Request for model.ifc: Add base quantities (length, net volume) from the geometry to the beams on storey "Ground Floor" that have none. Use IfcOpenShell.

First a look at what the model holds.

```python
import ifcopenshell
import ifcopenshell.util.element
import ifcopenshell.util.unit

model = ifcopenshell.open("model.ifc")
print(model.schema)
for unit_type in ("LENGTHUNIT", "AREAUNIT", "VOLUMEUNIT"):
    print(unit_type, ifcopenshell.util.unit.calculate_unit_scale(model, unit_type))
storey = next(s for s in model.by_type("IfcBuildingStorey") if s.Name == "Ground Floor")
beams = [e for e in ifcopenshell.util.element.get_decomposition(storey) if e.is_a("IfcBeam")]
for e in sorted(beams, key=lambda e: e.id()):
    print(e.id(), e.is_a(), e.Name, list(ifcopenshell.util.element.get_psets(e, qtos_only=True)), sep=" | ")
```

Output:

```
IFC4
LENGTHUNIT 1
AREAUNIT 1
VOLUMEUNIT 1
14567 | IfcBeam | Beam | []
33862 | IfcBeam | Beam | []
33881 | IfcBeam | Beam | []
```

```python
import ifcopenshell
import ifcopenshell.api.pset
import ifcopenshell.geom
import ifcopenshell.util.element
import ifcopenshell.util.shape
import ifcopenshell.util.unit

model = ifcopenshell.open("model.ifc")
unit_scale = ifcopenshell.util.unit.calculate_unit_scale(model)
volume_scale = ifcopenshell.util.unit.calculate_unit_scale(model, "VOLUMEUNIT")
settings = ifcopenshell.geom.settings()

storey = next(s for s in model.by_type("IfcBuildingStorey") if s.Name == "Ground Floor")
beams = [e for e in ifcopenshell.util.element.get_decomposition(storey) if e.is_a("IfcBeam")]

for e in sorted(beams, key=lambda e: e.id()):
    if ifcopenshell.util.element.get_psets(e, qtos_only=True, should_inherit=False):
        continue
    # Geometry comes back in metres, in the element's own axes.
    shape = ifcopenshell.geom.create_shape(settings, e)
    values = {
        "Length": ifcopenshell.util.shape.get_max_xyz(shape.geometry) / unit_scale,
        "NetVolume": ifcopenshell.util.shape.get_volume(shape.geometry) / volume_scale,
    }
    qto = ifcopenshell.api.pset.add_qto(model, product=e, name="Qto_BeamBaseQuantities")
    ifcopenshell.api.pset.edit_qto(model, qto=qto, properties=values)
    print(e.id(), {k: round(v, 3) for k, v in values.items()})

model.write("model_rev.ifc")
```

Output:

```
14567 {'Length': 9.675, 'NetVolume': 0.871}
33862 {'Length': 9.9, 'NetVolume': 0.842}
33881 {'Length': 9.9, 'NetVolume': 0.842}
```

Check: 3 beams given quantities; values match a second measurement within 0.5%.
